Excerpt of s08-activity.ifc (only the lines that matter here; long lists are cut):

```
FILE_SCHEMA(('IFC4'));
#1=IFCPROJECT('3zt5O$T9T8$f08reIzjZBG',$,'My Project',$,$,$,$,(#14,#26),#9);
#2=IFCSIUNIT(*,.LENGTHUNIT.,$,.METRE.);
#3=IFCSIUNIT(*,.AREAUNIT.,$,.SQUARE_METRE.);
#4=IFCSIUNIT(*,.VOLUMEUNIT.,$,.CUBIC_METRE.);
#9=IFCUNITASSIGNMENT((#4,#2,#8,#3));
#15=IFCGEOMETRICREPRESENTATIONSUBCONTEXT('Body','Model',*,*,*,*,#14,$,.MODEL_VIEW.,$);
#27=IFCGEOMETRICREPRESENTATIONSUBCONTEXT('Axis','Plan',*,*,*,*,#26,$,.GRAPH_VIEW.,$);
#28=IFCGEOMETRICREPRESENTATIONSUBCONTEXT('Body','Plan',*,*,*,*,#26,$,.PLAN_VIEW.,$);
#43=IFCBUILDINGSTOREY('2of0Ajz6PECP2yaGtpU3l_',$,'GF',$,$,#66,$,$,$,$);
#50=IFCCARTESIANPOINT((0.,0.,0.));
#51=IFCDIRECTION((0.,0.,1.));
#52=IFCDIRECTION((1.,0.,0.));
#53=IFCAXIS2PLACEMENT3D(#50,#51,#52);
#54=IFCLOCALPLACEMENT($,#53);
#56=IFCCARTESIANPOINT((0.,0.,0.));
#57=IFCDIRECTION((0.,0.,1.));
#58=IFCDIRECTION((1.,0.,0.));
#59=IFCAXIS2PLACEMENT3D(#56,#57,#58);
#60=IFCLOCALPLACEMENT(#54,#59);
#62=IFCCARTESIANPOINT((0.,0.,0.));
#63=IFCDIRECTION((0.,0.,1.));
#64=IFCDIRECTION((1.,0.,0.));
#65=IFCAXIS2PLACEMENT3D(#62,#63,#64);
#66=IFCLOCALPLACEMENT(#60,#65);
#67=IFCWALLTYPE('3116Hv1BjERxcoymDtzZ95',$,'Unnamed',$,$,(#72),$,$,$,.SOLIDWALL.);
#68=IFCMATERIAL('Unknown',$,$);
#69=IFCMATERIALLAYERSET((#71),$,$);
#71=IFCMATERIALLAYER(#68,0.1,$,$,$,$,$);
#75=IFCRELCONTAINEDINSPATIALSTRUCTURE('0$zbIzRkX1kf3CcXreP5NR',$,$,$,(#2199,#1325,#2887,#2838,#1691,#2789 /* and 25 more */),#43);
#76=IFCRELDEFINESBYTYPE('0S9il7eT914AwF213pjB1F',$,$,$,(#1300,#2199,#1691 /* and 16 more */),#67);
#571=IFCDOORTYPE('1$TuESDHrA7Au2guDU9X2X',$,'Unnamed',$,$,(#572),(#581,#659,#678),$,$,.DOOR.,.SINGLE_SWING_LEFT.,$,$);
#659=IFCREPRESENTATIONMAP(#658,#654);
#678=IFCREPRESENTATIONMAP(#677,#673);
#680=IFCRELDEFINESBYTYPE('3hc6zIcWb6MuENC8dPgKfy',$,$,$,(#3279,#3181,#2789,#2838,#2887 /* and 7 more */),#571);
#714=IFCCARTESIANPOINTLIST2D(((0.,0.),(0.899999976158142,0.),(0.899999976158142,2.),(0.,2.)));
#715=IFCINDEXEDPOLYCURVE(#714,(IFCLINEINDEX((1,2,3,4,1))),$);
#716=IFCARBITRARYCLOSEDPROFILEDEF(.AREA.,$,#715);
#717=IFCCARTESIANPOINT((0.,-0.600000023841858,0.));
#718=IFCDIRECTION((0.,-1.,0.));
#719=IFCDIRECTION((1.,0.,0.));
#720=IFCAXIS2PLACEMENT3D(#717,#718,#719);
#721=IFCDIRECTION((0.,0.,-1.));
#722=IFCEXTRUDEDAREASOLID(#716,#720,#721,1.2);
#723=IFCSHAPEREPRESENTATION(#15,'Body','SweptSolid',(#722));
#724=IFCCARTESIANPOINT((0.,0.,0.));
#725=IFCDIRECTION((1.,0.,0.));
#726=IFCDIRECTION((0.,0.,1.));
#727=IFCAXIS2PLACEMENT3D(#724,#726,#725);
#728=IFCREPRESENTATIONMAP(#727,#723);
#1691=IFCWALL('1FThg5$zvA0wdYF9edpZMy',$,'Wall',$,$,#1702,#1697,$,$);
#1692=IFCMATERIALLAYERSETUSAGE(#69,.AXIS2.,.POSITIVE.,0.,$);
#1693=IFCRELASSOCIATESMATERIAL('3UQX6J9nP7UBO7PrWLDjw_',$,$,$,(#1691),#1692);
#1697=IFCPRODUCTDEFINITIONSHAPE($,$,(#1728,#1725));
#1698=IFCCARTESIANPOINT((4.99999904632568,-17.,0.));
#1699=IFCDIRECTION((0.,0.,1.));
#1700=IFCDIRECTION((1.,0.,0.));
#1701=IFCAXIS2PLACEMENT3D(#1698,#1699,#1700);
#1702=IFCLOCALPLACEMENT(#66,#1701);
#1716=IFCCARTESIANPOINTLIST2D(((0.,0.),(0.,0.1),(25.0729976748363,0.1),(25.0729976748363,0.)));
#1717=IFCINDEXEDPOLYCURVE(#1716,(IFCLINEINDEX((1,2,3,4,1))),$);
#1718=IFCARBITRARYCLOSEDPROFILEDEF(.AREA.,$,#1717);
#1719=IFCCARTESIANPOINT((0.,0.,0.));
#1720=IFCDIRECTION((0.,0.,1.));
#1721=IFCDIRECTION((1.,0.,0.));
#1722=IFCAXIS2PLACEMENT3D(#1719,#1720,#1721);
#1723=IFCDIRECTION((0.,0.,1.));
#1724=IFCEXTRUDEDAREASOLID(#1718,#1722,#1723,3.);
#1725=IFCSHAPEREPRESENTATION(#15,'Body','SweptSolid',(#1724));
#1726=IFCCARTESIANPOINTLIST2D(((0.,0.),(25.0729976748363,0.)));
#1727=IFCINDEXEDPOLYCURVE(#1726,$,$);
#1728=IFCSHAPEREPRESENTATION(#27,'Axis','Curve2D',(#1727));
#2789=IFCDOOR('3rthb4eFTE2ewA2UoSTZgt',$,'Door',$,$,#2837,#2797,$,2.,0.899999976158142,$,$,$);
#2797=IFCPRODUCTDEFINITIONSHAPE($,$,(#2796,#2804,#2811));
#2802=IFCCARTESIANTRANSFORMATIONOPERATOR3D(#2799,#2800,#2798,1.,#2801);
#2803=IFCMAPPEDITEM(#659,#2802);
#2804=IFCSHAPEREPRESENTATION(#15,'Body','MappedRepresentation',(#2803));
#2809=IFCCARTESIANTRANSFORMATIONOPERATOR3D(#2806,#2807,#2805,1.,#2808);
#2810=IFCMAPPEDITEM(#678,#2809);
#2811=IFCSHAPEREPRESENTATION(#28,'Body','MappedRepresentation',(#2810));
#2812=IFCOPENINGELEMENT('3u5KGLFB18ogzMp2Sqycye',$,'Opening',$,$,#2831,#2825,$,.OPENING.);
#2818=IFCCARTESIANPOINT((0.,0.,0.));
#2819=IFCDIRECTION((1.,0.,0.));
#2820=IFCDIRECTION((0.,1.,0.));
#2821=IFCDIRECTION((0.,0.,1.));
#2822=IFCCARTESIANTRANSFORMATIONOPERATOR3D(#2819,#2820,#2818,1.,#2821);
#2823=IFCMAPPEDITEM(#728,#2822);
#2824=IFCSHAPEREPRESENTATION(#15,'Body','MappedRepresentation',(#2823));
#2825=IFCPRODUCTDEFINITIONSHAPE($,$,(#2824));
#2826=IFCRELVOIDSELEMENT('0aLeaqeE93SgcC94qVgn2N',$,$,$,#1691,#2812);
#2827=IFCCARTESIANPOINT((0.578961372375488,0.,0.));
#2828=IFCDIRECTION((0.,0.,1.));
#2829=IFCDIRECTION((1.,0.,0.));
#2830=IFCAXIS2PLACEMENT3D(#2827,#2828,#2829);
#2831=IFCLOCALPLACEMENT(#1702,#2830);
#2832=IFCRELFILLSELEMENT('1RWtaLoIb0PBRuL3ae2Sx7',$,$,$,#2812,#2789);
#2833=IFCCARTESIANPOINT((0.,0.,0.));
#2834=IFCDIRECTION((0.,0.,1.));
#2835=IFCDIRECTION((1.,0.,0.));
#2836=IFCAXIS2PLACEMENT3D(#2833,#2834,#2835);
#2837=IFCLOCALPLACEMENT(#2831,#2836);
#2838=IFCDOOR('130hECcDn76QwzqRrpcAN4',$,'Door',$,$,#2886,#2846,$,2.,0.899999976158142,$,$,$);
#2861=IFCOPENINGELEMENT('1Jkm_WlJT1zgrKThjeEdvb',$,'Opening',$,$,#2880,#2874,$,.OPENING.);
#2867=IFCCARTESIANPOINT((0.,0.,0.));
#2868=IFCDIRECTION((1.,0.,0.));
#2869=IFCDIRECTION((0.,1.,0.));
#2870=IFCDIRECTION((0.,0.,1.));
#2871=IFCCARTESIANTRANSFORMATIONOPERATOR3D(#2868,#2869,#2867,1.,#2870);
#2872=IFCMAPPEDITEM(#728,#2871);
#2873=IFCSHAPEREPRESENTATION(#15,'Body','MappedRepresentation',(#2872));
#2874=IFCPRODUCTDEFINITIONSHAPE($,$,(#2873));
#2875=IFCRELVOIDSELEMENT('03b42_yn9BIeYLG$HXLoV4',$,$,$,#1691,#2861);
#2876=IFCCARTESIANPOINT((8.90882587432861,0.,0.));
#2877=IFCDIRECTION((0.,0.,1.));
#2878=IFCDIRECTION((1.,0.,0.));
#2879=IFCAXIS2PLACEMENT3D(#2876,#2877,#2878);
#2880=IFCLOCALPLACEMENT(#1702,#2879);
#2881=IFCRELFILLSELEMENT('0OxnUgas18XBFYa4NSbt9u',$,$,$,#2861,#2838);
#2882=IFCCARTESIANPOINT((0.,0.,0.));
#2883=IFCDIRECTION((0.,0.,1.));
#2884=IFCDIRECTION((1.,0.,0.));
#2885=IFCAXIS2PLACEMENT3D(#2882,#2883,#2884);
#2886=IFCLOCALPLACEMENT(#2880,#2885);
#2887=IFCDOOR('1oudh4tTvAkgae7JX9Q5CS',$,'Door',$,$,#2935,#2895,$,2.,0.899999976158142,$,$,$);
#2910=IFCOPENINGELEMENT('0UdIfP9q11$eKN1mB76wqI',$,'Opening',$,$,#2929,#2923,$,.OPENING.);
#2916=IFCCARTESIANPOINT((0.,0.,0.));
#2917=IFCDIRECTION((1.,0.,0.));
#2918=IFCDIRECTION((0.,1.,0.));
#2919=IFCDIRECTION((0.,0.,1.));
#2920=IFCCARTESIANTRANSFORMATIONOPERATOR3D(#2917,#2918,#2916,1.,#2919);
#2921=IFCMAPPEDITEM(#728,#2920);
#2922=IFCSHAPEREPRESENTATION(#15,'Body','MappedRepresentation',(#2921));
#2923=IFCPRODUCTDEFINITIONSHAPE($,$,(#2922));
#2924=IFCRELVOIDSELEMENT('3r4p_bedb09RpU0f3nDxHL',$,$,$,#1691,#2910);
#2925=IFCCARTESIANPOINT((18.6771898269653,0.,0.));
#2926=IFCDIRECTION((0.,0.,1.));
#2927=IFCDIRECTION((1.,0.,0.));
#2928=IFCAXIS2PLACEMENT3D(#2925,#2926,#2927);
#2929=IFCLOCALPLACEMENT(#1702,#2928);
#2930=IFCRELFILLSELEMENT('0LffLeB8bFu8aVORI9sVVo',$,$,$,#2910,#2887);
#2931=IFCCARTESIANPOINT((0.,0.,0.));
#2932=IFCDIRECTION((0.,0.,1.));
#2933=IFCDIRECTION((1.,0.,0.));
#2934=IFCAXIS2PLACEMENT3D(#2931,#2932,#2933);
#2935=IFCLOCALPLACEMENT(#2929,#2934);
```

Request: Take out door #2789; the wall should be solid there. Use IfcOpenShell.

```python
import ifcopenshell
import ifcopenshell.api.feature
import ifcopenshell.api.root
import ifcopenshell.geom
import ifcopenshell.util.shape

model = ifcopenshell.open("s08-activity.ifc")
settings = ifcopenshell.geom.settings()


def volume(element):
    """Net volume in cubic metres, openings subtracted."""
    shape = ifcopenshell.geom.create_shape(settings, element)
    return ifcopenshell.util.shape.get_volume(shape.geometry)


door = model.by_guid("3rthb4eFTE2ewA2UoSTZgt")
opening = door.FillsVoids[0].RelatingOpeningElement
wall = opening.VoidsElements[0].RelatingBuildingElement
before = volume(wall)

ifcopenshell.api.root.remove_product(model, product=door)
ifcopenshell.api.feature.remove_feature(model, feature=opening)

after = volume(wall)

print(f"wall volume {before:.3f} -> {after:.3f} m3")

model.write("s08-activity_rev.ifc")
```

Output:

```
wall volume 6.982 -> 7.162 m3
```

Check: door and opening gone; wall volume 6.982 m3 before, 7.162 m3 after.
